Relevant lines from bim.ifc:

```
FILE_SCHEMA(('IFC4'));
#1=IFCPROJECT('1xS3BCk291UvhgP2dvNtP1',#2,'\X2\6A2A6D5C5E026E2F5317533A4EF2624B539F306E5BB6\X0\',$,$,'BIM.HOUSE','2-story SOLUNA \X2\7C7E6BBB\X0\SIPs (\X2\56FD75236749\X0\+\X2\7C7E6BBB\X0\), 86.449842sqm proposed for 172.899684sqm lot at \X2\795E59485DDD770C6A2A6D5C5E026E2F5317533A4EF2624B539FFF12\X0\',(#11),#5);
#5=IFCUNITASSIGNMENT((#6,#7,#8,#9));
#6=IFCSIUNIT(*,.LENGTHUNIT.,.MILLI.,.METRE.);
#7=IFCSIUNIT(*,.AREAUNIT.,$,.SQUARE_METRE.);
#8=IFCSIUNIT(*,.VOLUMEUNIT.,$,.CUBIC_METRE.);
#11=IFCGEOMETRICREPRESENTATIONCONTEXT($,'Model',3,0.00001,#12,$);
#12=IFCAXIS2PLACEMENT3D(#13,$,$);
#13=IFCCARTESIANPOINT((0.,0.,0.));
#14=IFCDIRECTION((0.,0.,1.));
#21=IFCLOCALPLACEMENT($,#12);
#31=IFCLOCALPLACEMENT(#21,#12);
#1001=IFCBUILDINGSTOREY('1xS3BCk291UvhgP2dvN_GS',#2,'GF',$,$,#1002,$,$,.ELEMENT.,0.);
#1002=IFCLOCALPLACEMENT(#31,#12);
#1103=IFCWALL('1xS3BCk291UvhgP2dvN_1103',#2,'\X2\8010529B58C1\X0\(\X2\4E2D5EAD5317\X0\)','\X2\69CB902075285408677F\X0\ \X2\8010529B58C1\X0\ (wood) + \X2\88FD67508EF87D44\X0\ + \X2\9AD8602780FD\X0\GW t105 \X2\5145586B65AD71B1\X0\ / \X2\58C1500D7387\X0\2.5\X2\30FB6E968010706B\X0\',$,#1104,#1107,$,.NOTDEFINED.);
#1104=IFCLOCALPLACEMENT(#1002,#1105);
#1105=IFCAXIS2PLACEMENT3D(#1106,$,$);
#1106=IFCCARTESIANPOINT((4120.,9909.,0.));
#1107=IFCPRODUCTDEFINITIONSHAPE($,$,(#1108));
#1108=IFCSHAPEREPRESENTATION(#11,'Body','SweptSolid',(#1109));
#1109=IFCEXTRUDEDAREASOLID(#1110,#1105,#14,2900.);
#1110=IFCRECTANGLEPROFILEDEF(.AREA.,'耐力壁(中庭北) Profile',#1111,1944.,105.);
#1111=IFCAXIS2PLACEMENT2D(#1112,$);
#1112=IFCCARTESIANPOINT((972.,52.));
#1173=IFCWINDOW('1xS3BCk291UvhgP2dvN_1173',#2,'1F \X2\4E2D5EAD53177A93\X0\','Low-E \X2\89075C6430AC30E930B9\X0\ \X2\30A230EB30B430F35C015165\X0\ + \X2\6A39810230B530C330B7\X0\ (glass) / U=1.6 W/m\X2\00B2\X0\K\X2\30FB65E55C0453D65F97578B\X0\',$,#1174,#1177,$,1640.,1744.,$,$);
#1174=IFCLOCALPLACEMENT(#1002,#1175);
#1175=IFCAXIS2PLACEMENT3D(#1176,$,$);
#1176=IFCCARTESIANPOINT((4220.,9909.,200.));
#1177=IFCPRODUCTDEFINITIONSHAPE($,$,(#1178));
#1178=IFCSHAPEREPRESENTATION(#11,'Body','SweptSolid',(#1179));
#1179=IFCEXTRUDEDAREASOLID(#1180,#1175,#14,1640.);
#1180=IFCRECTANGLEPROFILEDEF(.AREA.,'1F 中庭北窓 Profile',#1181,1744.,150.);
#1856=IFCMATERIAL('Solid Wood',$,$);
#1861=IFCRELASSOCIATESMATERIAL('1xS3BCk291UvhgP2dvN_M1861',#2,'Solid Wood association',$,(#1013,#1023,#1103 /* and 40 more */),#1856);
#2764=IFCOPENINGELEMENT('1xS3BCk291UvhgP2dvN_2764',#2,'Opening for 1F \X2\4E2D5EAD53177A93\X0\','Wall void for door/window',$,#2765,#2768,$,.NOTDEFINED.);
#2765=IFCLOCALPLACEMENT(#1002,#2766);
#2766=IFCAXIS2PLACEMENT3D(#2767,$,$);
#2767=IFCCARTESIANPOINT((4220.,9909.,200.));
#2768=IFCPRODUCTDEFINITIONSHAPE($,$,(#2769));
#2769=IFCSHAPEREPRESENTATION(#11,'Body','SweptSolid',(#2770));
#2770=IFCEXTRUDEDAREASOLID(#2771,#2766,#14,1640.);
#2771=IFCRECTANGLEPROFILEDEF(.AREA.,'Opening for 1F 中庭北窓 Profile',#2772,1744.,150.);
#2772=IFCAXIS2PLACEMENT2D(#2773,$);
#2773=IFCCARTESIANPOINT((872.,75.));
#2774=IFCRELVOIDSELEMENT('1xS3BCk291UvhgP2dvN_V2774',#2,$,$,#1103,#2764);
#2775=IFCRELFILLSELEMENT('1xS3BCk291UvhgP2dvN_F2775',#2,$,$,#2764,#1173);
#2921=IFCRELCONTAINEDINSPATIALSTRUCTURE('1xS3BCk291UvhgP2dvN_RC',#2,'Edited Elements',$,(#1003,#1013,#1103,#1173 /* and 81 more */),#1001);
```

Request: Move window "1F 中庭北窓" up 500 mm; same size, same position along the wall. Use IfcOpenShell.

```python
import numpy as np
import ifcopenshell
import ifcopenshell.api.geometry
import ifcopenshell.util.placement
import ifcopenshell.util.unit

model = ifcopenshell.open("bim.ifc")
unit_scale = ifcopenshell.util.unit.calculate_unit_scale(model)

window = model.by_guid("1xS3BCk291UvhgP2dvN_1173")
opening = window.FillsVoids[0].RelatingOpeningElement
dz = 0.5 / unit_scale

shift = np.array([0.0, 0.0, dz])
# The window is not placed relative to its opening, so move both.
for product in (opening, window):
    matrix = ifcopenshell.util.placement.get_local_placement(product.ObjectPlacement)
    matrix[:3, 3] += shift
    ifcopenshell.api.geometry.edit_object_placement(model, product=product, matrix=matrix, is_si=False)

print(f"moved by {dz * unit_scale:+.3f} m")

model.write("bim_edited.ifc")
```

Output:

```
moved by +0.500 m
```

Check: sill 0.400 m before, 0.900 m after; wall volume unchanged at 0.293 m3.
